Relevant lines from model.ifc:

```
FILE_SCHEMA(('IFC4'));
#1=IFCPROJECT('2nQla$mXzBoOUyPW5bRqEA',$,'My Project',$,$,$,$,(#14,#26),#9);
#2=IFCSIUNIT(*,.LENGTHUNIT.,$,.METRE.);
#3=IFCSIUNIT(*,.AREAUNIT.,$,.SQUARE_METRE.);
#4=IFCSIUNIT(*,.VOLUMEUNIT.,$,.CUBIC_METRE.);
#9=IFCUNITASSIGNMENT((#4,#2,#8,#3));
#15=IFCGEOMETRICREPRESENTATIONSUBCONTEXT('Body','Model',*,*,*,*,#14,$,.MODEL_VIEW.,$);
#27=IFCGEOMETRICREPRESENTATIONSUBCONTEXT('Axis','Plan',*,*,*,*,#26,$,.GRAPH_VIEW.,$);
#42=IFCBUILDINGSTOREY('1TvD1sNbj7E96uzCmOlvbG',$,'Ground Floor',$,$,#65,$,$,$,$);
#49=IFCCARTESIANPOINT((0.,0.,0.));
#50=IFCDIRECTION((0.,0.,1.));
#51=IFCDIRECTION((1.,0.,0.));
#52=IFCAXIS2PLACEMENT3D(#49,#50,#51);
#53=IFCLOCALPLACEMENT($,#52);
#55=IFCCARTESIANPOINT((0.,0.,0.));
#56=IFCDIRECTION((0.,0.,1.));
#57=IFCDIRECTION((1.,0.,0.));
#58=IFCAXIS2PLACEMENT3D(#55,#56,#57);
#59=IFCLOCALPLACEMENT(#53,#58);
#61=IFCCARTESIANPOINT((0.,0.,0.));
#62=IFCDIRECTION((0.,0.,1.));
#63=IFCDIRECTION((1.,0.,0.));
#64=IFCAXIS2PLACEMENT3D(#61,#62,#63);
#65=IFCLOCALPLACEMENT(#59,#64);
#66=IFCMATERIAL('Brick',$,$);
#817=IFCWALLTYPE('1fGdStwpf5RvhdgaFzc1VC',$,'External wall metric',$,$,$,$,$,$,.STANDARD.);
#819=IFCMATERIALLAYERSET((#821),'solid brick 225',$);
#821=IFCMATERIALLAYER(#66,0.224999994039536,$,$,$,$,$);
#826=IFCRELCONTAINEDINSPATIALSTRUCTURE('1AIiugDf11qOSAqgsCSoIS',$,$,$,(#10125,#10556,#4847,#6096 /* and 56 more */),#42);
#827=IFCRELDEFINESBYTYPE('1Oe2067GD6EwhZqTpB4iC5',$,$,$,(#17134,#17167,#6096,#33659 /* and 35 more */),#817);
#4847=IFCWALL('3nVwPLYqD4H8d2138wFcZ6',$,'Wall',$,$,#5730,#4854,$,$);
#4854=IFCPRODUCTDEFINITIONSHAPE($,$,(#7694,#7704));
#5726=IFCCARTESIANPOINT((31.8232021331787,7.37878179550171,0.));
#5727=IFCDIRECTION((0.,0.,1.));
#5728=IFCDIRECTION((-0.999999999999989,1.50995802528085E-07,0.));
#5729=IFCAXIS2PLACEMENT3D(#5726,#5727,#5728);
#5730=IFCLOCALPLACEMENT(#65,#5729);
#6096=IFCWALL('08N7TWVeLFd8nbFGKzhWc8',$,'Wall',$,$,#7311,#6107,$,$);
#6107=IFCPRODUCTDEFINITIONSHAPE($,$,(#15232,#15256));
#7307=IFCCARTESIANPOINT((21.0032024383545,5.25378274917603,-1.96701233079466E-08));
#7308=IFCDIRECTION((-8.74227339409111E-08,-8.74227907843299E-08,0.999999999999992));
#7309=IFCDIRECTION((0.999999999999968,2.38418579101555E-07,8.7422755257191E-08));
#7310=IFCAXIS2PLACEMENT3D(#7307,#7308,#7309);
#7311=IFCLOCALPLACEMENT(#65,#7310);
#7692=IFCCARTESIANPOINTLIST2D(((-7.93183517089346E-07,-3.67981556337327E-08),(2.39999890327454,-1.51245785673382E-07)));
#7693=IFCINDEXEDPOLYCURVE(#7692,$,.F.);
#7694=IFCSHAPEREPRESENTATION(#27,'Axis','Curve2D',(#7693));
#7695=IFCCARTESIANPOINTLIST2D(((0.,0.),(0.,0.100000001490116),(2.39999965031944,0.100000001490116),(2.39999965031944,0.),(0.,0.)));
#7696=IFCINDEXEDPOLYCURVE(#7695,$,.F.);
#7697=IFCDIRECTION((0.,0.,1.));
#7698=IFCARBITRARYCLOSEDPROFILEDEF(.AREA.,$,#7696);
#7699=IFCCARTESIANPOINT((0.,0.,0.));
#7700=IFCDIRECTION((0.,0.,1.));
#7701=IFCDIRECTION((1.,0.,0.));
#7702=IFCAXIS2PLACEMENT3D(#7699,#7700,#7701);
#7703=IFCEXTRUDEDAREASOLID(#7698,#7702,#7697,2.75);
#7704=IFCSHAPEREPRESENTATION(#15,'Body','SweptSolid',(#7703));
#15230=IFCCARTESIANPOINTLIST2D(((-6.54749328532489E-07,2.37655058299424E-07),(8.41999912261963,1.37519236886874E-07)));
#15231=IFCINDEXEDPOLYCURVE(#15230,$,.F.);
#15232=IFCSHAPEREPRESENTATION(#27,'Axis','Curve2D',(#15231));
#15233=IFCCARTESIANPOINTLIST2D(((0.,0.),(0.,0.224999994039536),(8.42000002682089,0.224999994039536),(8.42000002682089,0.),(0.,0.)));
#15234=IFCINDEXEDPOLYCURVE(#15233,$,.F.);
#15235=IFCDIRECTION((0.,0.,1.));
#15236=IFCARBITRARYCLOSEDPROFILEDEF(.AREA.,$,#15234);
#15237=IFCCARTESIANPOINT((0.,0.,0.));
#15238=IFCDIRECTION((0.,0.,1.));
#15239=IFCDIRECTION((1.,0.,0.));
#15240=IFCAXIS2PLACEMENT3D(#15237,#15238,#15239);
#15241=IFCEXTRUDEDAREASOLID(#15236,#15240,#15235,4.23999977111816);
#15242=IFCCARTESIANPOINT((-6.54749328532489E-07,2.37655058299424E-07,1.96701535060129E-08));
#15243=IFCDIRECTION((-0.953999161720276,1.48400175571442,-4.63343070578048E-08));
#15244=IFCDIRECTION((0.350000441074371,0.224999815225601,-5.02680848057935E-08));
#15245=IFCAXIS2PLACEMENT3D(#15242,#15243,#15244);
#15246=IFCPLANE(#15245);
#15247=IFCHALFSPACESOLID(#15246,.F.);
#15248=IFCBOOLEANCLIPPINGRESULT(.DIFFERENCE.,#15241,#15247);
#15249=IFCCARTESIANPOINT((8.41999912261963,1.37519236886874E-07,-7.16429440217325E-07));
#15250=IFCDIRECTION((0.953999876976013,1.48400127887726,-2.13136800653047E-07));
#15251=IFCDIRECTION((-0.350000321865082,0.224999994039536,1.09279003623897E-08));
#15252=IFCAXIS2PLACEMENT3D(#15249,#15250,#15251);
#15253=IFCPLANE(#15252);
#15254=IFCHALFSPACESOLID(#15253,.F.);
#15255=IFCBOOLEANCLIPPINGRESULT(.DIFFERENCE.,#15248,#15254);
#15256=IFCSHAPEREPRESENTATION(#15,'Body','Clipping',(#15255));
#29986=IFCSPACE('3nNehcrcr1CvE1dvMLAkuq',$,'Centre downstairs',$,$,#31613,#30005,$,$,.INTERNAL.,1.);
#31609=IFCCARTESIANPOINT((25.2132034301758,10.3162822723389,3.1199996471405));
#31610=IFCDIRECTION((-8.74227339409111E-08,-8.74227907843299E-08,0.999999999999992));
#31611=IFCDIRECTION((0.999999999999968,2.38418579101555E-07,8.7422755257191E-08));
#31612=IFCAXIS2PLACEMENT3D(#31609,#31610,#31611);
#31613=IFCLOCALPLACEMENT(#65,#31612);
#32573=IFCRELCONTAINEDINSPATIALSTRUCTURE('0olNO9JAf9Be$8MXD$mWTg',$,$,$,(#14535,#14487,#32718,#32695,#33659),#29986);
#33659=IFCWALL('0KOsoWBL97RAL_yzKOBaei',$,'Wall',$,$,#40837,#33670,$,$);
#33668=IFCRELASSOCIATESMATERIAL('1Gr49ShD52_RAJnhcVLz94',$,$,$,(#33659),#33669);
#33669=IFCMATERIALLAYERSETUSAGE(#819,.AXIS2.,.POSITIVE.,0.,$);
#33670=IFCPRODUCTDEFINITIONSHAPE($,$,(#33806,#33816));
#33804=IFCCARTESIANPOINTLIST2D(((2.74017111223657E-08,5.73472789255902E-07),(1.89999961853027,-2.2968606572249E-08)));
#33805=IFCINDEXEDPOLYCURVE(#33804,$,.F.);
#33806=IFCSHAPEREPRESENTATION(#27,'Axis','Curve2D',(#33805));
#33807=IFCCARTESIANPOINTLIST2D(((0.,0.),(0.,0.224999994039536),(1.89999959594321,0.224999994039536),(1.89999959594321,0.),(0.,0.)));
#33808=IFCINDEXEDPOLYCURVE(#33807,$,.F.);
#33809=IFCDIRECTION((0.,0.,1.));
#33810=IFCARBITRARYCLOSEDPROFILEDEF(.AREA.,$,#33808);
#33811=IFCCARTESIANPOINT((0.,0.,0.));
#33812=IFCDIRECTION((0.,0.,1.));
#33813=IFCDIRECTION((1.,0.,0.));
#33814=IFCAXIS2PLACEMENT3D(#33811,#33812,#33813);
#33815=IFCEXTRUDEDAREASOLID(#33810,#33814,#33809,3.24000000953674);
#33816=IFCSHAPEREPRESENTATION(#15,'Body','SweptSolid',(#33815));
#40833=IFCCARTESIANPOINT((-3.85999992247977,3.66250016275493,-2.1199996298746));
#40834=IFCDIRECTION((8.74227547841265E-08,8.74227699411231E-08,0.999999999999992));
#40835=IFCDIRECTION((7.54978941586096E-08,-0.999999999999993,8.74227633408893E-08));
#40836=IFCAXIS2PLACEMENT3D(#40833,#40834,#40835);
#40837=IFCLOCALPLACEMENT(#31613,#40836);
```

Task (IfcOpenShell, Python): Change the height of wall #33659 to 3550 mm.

```python
import ifcopenshell
import ifcopenshell.geom
import ifcopenshell.util.representation
import ifcopenshell.util.shape

model = ifcopenshell.open("model.ifc")
settings = ifcopenshell.geom.settings()


def volume(element):
    """Net volume in cubic metres, openings subtracted."""
    shape = ifcopenshell.geom.create_shape(settings, element)
    return ifcopenshell.util.shape.get_volume(shape.geometry)


wall = model.by_id(33659)
before = volume(wall)

body = ifcopenshell.util.representation.get_representation(wall, "Model", "Body")
solid = body.Items[0]
old_height = solid.Depth
solid.Depth = 3.55
after = volume(wall)

print(f"height {old_height:g} -> {solid.Depth:g}, volume {before:.3f} -> {after:.3f} m3")

model.write("model_edited.ifc")
```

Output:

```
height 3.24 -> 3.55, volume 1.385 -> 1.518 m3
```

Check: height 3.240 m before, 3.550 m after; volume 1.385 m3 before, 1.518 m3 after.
